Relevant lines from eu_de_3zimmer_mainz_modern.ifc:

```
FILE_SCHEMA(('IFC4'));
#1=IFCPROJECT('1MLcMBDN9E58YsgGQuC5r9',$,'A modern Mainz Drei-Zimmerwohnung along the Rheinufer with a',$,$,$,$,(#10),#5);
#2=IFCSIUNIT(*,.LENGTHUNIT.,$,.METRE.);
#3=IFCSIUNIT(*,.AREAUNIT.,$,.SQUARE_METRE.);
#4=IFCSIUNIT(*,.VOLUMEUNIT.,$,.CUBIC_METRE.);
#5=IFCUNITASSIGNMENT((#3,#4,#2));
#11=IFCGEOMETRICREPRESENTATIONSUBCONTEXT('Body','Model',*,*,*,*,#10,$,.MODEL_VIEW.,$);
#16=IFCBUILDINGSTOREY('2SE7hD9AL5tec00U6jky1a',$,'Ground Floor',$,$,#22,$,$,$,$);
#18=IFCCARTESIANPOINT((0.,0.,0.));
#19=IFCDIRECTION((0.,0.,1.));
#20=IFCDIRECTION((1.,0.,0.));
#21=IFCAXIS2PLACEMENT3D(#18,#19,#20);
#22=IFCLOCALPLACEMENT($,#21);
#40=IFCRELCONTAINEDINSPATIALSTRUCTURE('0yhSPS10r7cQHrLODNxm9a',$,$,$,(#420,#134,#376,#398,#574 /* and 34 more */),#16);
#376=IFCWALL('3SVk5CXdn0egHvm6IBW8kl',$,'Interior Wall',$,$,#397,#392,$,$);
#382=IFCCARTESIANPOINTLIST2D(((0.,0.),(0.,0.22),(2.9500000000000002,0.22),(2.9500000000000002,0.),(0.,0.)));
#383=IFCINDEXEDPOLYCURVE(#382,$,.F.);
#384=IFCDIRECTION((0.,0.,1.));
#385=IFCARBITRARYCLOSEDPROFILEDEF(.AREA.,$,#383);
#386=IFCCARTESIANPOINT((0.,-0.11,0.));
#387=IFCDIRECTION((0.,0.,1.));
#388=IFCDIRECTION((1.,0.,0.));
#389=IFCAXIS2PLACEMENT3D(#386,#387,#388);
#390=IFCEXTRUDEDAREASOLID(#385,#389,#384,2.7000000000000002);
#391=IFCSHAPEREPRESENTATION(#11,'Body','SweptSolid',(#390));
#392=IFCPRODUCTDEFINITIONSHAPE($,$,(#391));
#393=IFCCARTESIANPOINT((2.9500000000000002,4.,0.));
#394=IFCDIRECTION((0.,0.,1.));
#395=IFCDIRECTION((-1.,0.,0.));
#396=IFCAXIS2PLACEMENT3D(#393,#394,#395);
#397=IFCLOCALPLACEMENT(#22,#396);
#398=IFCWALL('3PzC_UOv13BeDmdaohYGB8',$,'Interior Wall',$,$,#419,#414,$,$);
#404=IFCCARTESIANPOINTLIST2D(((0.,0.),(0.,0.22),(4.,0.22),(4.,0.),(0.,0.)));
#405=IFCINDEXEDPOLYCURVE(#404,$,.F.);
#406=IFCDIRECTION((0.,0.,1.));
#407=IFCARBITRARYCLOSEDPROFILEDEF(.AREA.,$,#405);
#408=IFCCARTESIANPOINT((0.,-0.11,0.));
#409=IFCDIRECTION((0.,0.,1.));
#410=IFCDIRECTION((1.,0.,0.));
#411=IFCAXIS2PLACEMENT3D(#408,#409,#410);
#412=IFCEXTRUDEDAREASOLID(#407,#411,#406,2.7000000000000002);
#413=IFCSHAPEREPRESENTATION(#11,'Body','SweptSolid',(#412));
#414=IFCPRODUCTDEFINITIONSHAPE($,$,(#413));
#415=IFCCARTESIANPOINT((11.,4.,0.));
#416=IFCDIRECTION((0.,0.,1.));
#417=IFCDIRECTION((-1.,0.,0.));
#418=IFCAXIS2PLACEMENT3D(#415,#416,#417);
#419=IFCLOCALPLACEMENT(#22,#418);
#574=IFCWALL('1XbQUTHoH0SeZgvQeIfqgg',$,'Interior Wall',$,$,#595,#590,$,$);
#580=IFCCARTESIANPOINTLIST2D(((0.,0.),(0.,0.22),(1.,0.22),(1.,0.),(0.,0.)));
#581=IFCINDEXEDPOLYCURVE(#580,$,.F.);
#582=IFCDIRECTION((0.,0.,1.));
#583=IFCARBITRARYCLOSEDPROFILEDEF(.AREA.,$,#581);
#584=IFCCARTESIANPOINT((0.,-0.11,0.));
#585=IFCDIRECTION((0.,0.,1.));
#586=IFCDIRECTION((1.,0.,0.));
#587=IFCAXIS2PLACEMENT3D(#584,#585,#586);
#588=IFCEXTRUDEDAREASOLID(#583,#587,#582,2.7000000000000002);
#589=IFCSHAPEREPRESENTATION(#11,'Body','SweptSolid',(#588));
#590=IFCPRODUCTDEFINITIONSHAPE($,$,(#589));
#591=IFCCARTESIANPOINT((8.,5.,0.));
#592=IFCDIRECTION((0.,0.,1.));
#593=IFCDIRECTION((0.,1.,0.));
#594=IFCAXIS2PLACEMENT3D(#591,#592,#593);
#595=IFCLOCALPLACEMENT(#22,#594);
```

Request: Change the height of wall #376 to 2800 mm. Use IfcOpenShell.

```python
import ifcopenshell
import ifcopenshell.geom
import ifcopenshell.util.representation
import ifcopenshell.util.shape

model = ifcopenshell.open("eu_de_3zimmer_mainz_modern.ifc")
settings = ifcopenshell.geom.settings()


def volume(element):
    """Net volume in cubic metres, openings subtracted."""
    shape = ifcopenshell.geom.create_shape(settings, element)
    return ifcopenshell.util.shape.get_volume(shape.geometry)


wall = model.by_guid("3SVk5CXdn0egHvm6IBW8kl")
before = volume(wall)

body = ifcopenshell.util.representation.get_representation(wall, "Model", "Body")
solid = body.Items[0]
old_height = solid.Depth
solid.Depth = 2.8
after = volume(wall)

print(f"height {old_height:g} -> {solid.Depth:g}, volume {before:.3f} -> {after:.3f} m3")

model.write("eu_de_3zimmer_mainz_modern_rev.ifc")
```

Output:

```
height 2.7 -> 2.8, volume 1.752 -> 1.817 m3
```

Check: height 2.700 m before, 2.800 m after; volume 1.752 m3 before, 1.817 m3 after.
